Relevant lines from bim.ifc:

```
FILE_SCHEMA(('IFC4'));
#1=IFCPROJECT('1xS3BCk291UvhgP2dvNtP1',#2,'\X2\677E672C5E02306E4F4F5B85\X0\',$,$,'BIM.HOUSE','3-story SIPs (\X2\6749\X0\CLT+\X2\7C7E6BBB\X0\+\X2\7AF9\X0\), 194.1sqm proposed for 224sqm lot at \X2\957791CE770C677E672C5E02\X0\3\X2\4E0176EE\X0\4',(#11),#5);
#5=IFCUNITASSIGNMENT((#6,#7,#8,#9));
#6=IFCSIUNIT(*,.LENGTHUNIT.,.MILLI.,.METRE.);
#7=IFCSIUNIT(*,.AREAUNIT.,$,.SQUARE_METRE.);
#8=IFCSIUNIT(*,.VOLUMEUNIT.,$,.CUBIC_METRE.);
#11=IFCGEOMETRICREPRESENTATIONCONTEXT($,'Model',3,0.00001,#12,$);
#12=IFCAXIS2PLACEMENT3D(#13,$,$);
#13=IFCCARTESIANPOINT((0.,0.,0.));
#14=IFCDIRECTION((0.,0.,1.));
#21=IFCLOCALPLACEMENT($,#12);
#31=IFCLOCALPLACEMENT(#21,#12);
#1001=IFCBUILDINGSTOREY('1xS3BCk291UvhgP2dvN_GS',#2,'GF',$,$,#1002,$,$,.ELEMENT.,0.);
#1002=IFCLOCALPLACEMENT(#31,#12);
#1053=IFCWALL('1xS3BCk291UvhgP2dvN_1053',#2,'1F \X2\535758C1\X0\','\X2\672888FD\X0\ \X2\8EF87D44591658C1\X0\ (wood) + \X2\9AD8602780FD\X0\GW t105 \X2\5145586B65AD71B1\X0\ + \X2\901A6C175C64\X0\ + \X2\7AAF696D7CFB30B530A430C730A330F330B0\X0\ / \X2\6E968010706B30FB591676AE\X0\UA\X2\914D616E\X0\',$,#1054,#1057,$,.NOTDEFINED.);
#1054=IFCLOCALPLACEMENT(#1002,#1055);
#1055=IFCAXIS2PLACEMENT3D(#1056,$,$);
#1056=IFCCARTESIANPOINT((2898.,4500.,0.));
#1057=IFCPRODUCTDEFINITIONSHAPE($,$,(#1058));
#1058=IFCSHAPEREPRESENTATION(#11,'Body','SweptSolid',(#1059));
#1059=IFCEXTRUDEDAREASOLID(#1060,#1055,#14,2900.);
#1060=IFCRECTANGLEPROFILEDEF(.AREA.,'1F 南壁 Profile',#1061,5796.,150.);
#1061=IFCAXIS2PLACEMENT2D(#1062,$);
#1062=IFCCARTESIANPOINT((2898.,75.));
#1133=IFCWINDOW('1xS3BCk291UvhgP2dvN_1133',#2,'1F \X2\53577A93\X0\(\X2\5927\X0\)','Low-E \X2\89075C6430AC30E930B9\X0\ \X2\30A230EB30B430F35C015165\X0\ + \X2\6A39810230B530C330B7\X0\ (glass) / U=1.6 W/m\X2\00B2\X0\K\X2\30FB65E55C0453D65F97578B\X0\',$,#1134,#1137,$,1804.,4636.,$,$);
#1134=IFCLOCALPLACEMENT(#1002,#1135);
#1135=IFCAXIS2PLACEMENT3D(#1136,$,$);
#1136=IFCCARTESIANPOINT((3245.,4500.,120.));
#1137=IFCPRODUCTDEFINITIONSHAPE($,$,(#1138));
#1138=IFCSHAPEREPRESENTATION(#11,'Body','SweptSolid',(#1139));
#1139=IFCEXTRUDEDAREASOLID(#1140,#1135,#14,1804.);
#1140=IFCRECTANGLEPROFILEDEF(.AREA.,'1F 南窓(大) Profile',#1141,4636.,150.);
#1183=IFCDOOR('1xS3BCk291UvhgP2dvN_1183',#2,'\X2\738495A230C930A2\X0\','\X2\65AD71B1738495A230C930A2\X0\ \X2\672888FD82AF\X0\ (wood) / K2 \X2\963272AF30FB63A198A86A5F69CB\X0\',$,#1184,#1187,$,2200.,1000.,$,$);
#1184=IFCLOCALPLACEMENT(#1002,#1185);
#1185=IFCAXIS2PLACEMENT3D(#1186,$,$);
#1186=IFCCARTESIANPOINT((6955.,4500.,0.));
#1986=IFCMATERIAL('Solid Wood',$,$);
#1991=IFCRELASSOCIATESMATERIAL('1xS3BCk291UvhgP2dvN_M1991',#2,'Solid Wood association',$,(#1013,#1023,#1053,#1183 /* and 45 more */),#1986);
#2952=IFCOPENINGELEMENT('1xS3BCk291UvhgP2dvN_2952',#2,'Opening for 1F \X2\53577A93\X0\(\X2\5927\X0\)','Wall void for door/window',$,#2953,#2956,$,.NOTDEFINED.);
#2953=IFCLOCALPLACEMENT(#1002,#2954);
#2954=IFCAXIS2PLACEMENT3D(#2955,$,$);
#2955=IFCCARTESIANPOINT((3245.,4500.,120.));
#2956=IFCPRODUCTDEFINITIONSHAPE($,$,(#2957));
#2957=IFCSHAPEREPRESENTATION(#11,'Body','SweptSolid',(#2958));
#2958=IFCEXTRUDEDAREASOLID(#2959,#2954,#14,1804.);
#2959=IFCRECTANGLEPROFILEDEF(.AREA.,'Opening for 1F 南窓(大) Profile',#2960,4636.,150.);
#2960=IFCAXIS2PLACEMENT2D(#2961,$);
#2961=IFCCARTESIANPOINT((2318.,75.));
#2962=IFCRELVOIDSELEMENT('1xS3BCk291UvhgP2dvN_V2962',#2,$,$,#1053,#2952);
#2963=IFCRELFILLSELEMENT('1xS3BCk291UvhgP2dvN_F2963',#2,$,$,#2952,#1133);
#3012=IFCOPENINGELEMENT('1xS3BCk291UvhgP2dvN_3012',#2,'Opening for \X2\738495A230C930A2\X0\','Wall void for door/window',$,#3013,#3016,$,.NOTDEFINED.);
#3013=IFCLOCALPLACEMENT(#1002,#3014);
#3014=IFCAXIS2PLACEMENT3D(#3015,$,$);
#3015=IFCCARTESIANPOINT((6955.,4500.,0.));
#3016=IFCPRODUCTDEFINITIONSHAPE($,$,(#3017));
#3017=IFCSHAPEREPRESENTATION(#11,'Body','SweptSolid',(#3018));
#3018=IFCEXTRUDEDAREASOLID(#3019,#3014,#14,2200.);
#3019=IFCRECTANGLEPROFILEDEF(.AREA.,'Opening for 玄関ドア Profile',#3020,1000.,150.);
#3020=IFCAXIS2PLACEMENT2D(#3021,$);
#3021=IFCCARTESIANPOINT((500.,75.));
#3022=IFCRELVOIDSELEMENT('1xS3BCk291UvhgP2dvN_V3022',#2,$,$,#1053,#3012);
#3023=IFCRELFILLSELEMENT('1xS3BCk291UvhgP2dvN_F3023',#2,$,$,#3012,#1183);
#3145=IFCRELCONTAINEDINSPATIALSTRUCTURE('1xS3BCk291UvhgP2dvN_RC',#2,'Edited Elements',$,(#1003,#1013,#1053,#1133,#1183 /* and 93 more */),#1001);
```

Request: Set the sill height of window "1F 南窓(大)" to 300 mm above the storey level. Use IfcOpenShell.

```python
import numpy as np
import ifcopenshell
import ifcopenshell.api.geometry
import ifcopenshell.geom
import ifcopenshell.util.element
import ifcopenshell.util.placement
import ifcopenshell.util.shape
import ifcopenshell.util.unit

model = ifcopenshell.open("bim.ifc")
unit_scale = ifcopenshell.util.unit.calculate_unit_scale(model)

window = model.by_guid("1xS3BCk291UvhgP2dvN_1133")
opening = window.FillsVoids[0].RelatingOpeningElement
storey = ifcopenshell.util.element.get_container(window, ifc_class="IfcBuildingStorey")
level = ifcopenshell.util.placement.get_local_placement(storey.ObjectPlacement)[2, 3]

# The opening's origin need not be at the sill, so measure its lowest point.
shape = ifcopenshell.geom.create_shape(ifcopenshell.geom.settings(), opening)
bottom = ifcopenshell.util.shape.get_shape_bottom_elevation(shape, shape.geometry) / unit_scale
dz = level + 300.0 - bottom

shift = np.array([0.0, 0.0, dz])
# The window is not placed relative to its opening, so move both.
for product in (opening, window):
    matrix = ifcopenshell.util.placement.get_local_placement(product.ObjectPlacement)
    matrix[:3, 3] += shift
    ifcopenshell.api.geometry.edit_object_placement(model, product=product, matrix=matrix, is_si=False)

print(f"moved by {dz * unit_scale:+.3f} m")

model.write("bim_rev.ifc")
```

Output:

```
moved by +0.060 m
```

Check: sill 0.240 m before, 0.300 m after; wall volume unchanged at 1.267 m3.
